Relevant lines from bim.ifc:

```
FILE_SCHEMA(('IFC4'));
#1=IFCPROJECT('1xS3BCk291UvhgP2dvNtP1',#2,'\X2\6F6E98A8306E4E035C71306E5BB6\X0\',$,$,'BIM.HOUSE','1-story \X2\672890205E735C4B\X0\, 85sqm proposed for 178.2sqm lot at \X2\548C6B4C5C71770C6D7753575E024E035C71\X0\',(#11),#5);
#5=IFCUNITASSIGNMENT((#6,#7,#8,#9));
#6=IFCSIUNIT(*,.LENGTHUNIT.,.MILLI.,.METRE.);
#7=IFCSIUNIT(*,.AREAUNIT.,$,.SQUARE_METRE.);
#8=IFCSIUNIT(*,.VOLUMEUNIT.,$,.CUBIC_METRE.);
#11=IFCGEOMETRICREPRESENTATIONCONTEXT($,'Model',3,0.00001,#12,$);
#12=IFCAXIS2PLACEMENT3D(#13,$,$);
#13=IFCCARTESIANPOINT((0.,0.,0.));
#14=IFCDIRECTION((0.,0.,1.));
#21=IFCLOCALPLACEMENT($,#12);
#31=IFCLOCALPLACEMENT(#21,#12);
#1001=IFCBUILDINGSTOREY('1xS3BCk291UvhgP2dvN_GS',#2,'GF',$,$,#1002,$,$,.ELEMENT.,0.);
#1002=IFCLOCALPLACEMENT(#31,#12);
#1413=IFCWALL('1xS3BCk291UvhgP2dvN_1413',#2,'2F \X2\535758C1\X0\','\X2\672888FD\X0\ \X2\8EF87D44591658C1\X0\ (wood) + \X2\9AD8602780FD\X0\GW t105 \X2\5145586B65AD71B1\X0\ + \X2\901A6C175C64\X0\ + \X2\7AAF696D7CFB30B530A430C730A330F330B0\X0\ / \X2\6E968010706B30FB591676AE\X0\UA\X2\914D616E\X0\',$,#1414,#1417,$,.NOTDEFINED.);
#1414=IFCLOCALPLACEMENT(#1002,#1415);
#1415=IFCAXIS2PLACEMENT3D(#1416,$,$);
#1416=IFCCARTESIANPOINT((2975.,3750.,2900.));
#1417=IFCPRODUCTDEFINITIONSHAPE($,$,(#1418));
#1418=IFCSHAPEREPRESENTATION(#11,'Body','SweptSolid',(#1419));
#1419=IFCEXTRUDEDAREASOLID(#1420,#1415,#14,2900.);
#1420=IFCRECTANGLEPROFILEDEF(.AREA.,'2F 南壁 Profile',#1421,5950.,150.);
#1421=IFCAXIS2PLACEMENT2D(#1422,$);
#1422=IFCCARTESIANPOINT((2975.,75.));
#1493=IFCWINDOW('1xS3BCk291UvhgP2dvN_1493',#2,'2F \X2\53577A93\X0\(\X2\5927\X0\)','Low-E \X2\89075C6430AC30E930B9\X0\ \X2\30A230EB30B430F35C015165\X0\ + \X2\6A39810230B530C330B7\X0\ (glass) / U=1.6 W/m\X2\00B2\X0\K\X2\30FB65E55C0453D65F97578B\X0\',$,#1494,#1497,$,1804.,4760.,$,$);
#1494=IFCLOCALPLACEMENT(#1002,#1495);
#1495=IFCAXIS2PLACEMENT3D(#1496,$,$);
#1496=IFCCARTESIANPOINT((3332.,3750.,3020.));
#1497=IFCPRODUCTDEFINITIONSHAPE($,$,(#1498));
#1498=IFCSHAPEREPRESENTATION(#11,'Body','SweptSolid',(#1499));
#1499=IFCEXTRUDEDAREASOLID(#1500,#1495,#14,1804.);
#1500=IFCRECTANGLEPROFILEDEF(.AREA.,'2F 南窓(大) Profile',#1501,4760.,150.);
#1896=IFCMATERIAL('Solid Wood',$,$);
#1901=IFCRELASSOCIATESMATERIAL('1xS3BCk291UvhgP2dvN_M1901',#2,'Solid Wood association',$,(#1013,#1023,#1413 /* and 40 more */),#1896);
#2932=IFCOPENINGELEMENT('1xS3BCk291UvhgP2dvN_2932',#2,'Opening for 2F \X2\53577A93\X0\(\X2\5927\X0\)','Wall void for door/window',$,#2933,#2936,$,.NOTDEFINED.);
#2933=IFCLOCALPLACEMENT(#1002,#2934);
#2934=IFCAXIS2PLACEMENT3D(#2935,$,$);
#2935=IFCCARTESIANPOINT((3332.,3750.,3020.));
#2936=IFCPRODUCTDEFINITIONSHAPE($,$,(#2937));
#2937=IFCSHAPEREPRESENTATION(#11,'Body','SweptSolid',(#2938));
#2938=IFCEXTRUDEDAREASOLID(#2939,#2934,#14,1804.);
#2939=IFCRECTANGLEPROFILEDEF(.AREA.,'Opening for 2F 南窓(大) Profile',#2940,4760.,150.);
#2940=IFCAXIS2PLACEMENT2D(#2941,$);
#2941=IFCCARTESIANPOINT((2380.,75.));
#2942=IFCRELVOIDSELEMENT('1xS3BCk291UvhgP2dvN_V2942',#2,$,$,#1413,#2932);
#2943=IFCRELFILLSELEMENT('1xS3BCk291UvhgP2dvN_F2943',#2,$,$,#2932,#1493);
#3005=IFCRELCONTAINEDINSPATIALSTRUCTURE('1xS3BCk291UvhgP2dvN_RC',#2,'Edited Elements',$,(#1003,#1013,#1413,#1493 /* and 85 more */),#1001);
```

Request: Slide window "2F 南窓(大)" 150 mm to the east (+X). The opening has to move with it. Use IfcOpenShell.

```python
import ifcopenshell
import ifcopenshell.api.geometry
import ifcopenshell.util.placement

model = ifcopenshell.open("bim.ifc")

window = model.by_id(1493)
opening = window.FillsVoids[0].RelatingOpeningElement
wall = opening.VoidsElements[0].RelatingBuildingElement

wall_matrix = ifcopenshell.util.placement.get_local_placement(wall.ObjectPlacement)
shift = wall_matrix[:3, 0] * 150.0
before = ifcopenshell.util.placement.get_local_placement(window.ObjectPlacement)[:3, 3].copy()

# The window is not placed relative to its opening, so move both.
for product in (opening, window):
    matrix = ifcopenshell.util.placement.get_local_placement(product.ObjectPlacement)
    matrix[:3, 3] += shift
    ifcopenshell.api.geometry.edit_object_placement(model, product=product, matrix=matrix, is_si=False)

after = ifcopenshell.util.placement.get_local_placement(window.ObjectPlacement)[:3, 3]
print("window moved by", (after - before).round(3) + 0.0)

model.write("bim_edited.ifc")
```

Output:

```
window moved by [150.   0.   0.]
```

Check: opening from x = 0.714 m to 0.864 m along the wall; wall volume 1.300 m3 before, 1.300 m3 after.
